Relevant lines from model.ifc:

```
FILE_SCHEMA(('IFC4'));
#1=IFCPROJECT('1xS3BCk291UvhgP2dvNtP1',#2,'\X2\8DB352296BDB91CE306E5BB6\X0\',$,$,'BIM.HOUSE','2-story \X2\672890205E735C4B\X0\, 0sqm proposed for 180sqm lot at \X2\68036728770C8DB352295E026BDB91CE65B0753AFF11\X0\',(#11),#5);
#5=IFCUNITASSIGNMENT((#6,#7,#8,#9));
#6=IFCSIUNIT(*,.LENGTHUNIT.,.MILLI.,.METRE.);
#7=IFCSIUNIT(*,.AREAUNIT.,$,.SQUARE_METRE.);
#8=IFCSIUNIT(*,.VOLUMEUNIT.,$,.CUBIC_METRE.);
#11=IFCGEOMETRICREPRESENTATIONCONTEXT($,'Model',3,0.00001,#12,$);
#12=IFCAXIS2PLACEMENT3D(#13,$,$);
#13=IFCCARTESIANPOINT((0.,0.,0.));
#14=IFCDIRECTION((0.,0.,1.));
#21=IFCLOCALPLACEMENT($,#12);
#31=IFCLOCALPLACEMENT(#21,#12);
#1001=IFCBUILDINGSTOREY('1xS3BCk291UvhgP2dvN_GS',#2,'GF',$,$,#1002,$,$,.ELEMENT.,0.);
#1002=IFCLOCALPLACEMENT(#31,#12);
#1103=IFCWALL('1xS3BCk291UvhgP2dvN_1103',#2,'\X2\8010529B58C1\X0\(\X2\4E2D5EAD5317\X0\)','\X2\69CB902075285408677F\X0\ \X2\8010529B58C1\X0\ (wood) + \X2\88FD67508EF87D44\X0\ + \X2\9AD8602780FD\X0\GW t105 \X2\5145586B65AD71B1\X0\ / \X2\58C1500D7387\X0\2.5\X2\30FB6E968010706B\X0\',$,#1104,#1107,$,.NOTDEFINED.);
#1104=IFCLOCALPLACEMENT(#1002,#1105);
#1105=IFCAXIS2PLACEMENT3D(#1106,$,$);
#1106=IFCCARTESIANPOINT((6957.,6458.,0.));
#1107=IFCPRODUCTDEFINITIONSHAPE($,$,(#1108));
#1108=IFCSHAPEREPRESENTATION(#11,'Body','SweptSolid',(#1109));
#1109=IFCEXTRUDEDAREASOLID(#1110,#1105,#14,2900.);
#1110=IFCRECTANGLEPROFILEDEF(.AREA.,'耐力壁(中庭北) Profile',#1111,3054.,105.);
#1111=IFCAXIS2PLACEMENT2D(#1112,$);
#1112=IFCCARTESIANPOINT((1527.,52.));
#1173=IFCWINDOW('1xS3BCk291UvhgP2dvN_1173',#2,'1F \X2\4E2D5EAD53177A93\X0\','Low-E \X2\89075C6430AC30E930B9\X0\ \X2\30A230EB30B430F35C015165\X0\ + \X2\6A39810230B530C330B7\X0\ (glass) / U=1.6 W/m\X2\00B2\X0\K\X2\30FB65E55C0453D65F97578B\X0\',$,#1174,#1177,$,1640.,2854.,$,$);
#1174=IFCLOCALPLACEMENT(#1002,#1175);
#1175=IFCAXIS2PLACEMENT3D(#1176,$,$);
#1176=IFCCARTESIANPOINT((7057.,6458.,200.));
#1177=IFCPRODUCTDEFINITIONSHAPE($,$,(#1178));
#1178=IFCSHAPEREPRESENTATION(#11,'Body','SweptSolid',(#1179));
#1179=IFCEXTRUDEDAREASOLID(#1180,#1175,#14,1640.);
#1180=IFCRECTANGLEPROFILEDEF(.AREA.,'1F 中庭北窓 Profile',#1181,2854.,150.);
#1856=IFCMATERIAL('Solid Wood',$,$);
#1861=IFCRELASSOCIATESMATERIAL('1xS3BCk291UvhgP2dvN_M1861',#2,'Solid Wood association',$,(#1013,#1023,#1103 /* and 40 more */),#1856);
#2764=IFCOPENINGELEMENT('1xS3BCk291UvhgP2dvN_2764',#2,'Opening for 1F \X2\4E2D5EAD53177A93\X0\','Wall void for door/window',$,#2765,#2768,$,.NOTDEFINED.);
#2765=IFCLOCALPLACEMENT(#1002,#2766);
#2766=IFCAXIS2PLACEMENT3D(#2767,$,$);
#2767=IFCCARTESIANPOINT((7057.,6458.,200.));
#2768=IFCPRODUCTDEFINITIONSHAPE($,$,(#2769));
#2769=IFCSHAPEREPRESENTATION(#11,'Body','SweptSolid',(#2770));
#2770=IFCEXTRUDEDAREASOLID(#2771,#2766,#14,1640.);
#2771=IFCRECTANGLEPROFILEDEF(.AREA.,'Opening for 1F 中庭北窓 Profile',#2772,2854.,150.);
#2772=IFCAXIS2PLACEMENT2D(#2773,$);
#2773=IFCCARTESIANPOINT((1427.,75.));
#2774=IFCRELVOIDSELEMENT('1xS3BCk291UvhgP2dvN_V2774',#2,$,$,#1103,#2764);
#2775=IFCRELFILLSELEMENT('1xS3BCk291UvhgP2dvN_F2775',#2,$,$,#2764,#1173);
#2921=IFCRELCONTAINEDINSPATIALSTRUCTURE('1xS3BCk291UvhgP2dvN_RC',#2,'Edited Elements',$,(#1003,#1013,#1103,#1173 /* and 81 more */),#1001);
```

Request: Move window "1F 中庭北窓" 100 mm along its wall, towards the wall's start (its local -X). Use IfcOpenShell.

```python
import ifcopenshell
import ifcopenshell.api.geometry
import ifcopenshell.util.placement
import ifcopenshell.util.unit

model = ifcopenshell.open("model.ifc")
unit_scale = ifcopenshell.util.unit.calculate_unit_scale(model)

window = model.by_id(1173)
opening = window.FillsVoids[0].RelatingOpeningElement
wall = opening.VoidsElements[0].RelatingBuildingElement

wall_matrix = ifcopenshell.util.placement.get_local_placement(wall.ObjectPlacement)
shift = wall_matrix[:3, 0] * -0.1 / unit_scale
before = ifcopenshell.util.placement.get_local_placement(window.ObjectPlacement)[:3, 3].copy()

# The window is not placed relative to its opening, so move both.
for product in (opening, window):
    matrix = ifcopenshell.util.placement.get_local_placement(product.ObjectPlacement)
    matrix[:3, 3] += shift
    ifcopenshell.api.geometry.edit_object_placement(model, product=product, matrix=matrix, is_si=False)

after = ifcopenshell.util.placement.get_local_placement(window.ObjectPlacement)[:3, 3]
print("window moved by", (after - before).round(3) + 0.0)

model.write("model_updated.ifc")
```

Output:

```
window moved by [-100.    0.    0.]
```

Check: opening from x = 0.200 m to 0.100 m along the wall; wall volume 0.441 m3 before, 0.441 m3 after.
